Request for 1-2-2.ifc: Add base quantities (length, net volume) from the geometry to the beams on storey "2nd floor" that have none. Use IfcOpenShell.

First a look at what the model holds.

```python
import ifcopenshell
import ifcopenshell.util.element
import ifcopenshell.util.unit

model = ifcopenshell.open("1-2-2.ifc")
print(model.schema)
for unit_type in ("LENGTHUNIT", "AREAUNIT", "VOLUMEUNIT"):
    print(unit_type, ifcopenshell.util.unit.calculate_unit_scale(model, unit_type))
storey = next(s for s in model.by_type("IfcBuildingStorey") if s.Name == "2nd floor")
beams = [e for e in ifcopenshell.util.element.get_decomposition(storey) if e.is_a("IfcBeam")]
for e in sorted(beams, key=lambda e: e.id()):
    print(e.id(), e.is_a(), e.Name, list(ifcopenshell.util.element.get_psets(e, qtos_only=True)), sep=" | ")
```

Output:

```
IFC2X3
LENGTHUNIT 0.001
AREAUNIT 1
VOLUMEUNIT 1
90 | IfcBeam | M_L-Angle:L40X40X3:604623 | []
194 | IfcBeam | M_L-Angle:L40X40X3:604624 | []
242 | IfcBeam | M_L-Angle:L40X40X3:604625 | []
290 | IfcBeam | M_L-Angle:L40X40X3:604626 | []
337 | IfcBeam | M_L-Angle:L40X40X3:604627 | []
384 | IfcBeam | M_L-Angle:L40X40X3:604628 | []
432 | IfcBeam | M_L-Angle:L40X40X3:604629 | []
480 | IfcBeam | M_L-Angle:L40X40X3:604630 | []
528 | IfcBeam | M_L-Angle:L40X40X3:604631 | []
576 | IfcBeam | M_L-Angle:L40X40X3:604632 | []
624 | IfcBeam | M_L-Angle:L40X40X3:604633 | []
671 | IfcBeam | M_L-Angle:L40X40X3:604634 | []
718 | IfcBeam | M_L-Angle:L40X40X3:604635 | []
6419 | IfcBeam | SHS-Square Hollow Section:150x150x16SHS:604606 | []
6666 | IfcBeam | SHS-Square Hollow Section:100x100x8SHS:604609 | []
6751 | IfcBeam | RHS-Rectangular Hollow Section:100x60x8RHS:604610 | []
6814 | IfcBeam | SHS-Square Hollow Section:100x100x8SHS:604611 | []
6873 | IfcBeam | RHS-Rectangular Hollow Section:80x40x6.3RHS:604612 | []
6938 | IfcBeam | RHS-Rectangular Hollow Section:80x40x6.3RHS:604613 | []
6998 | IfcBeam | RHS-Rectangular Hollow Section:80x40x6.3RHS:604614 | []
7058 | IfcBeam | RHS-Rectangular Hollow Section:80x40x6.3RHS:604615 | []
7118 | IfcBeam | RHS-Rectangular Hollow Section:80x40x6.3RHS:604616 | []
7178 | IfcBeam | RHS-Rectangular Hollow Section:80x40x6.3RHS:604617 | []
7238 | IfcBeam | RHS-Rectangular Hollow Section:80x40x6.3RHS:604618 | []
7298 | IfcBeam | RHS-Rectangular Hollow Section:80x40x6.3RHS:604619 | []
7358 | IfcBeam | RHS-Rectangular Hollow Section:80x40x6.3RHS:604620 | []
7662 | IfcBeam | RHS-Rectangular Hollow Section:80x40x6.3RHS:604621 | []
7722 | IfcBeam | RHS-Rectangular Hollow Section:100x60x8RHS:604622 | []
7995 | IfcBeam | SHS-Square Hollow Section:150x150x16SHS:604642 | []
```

```python
import ifcopenshell
import ifcopenshell.api.pset
import ifcopenshell.geom
import ifcopenshell.util.element
import ifcopenshell.util.shape
import ifcopenshell.util.unit

model = ifcopenshell.open("1-2-2.ifc")
unit_scale = ifcopenshell.util.unit.calculate_unit_scale(model)
volume_scale = ifcopenshell.util.unit.calculate_unit_scale(model, "VOLUMEUNIT")
settings = ifcopenshell.geom.settings()

storey = next(s for s in model.by_type("IfcBuildingStorey") if s.Name == "2nd floor")
beams = [e for e in ifcopenshell.util.element.get_decomposition(storey) if e.is_a("IfcBeam")]

for e in sorted(beams, key=lambda e: e.id()):
    if ifcopenshell.util.element.get_psets(e, qtos_only=True, should_inherit=False):
        continue
    # Geometry comes back in metres, in the element's own axes.
    shape = ifcopenshell.geom.create_shape(settings, e)
    values = {
        "Length": ifcopenshell.util.shape.get_max_xyz(shape.geometry) / unit_scale,
        "NetVolume": ifcopenshell.util.shape.get_volume(shape.geometry) / volume_scale,
    }
    qto = ifcopenshell.api.pset.add_qto(model, product=e, name="BaseQuantities")
    ifcopenshell.api.pset.edit_qto(model, qto=qto, properties=values)
    print(e.id(), {k: round(v, 3) for k, v in values.items()})

model.write("1-2-2_v2.ifc")
```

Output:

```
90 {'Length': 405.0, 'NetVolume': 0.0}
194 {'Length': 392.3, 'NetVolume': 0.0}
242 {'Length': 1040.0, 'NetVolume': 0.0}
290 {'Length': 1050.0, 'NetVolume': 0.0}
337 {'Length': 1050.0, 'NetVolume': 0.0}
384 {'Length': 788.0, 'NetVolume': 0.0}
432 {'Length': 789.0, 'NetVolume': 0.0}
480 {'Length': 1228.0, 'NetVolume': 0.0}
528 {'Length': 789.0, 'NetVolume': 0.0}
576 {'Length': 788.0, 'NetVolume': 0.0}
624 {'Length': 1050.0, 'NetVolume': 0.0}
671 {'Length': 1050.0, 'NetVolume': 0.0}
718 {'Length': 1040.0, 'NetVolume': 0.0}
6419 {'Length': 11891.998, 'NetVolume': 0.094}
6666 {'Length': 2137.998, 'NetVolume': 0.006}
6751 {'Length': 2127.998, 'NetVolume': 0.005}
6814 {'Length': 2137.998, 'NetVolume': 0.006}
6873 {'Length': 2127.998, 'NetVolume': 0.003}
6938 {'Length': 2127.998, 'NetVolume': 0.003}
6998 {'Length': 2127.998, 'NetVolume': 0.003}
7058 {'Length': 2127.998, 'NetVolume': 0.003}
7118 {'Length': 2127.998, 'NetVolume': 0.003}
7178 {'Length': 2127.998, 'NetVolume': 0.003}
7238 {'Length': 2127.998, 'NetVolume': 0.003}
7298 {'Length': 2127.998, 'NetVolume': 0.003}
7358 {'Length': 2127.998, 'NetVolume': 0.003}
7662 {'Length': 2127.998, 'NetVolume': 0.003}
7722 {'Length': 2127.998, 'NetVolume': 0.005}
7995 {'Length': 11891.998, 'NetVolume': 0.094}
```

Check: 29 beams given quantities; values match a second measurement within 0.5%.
